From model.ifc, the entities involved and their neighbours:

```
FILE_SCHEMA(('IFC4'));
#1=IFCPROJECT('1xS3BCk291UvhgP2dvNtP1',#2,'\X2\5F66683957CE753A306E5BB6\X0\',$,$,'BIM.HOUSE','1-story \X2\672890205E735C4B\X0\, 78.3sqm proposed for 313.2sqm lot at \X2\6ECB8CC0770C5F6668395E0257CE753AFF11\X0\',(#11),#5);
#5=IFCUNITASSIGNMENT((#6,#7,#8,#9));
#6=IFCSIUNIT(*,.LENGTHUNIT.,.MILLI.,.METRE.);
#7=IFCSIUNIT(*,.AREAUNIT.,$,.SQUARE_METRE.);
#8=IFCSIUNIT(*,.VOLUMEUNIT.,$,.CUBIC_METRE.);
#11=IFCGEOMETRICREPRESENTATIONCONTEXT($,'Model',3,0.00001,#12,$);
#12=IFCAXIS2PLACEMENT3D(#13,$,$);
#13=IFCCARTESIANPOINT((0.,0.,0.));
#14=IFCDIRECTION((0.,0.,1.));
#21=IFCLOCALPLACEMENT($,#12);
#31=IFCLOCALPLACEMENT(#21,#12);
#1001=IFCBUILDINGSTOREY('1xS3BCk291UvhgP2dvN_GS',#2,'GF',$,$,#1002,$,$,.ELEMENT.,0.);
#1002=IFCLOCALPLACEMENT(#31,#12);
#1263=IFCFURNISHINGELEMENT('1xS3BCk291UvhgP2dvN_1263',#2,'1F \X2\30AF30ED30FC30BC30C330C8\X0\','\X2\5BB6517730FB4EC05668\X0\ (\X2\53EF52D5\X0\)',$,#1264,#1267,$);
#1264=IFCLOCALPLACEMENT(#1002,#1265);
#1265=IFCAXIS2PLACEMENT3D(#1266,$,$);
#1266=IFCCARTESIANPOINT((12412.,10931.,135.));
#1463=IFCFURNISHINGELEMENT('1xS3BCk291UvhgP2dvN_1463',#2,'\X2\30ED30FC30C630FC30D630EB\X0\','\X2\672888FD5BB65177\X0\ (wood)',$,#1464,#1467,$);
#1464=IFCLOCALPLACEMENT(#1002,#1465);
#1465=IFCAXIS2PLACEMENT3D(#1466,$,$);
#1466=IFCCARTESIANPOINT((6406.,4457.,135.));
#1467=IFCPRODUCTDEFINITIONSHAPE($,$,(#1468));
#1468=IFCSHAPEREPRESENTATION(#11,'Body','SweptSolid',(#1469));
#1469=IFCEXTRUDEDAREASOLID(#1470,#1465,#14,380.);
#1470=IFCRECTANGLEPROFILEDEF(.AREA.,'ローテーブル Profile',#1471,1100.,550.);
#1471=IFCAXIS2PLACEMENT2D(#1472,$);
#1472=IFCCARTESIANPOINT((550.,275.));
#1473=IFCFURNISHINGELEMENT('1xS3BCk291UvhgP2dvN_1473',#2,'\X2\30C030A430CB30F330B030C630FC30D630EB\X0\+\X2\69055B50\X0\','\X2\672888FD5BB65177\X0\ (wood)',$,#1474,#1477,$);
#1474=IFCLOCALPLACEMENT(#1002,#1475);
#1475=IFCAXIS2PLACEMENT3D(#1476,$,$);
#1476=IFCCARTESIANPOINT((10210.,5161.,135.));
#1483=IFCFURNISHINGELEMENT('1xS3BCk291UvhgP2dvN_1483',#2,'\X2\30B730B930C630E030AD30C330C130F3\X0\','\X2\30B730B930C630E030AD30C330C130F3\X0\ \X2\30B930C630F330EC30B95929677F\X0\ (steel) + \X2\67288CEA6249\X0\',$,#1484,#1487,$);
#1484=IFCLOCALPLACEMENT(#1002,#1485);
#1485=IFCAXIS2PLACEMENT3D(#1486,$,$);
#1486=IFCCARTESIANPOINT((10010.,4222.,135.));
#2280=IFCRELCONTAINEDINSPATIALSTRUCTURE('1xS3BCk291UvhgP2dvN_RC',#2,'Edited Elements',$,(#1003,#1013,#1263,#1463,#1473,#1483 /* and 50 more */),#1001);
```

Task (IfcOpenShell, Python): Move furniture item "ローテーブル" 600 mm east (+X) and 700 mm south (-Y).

```python
import ifcopenshell
import ifcopenshell.api.geometry
import ifcopenshell.util.placement
import ifcopenshell.util.unit

model = ifcopenshell.open("model.ifc")
unit_scale = ifcopenshell.util.unit.calculate_unit_scale(model)

item = model.by_guid("1xS3BCk291UvhgP2dvN_1463")
matrix = ifcopenshell.util.placement.get_local_placement(item.ObjectPlacement)
matrix[0, 3] += 0.6 / unit_scale
matrix[1, 3] -= 0.7 / unit_scale
ifcopenshell.api.geometry.edit_object_placement(model, product=item, matrix=matrix, is_si=False)

print(ifcopenshell.util.placement.get_local_placement(item.ObjectPlacement).round(3) + 0.0)

model.write("model_updated.ifc")
```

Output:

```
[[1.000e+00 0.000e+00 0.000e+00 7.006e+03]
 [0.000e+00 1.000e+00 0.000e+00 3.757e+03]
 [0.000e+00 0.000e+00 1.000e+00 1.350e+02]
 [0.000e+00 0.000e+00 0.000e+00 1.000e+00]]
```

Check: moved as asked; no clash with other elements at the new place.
